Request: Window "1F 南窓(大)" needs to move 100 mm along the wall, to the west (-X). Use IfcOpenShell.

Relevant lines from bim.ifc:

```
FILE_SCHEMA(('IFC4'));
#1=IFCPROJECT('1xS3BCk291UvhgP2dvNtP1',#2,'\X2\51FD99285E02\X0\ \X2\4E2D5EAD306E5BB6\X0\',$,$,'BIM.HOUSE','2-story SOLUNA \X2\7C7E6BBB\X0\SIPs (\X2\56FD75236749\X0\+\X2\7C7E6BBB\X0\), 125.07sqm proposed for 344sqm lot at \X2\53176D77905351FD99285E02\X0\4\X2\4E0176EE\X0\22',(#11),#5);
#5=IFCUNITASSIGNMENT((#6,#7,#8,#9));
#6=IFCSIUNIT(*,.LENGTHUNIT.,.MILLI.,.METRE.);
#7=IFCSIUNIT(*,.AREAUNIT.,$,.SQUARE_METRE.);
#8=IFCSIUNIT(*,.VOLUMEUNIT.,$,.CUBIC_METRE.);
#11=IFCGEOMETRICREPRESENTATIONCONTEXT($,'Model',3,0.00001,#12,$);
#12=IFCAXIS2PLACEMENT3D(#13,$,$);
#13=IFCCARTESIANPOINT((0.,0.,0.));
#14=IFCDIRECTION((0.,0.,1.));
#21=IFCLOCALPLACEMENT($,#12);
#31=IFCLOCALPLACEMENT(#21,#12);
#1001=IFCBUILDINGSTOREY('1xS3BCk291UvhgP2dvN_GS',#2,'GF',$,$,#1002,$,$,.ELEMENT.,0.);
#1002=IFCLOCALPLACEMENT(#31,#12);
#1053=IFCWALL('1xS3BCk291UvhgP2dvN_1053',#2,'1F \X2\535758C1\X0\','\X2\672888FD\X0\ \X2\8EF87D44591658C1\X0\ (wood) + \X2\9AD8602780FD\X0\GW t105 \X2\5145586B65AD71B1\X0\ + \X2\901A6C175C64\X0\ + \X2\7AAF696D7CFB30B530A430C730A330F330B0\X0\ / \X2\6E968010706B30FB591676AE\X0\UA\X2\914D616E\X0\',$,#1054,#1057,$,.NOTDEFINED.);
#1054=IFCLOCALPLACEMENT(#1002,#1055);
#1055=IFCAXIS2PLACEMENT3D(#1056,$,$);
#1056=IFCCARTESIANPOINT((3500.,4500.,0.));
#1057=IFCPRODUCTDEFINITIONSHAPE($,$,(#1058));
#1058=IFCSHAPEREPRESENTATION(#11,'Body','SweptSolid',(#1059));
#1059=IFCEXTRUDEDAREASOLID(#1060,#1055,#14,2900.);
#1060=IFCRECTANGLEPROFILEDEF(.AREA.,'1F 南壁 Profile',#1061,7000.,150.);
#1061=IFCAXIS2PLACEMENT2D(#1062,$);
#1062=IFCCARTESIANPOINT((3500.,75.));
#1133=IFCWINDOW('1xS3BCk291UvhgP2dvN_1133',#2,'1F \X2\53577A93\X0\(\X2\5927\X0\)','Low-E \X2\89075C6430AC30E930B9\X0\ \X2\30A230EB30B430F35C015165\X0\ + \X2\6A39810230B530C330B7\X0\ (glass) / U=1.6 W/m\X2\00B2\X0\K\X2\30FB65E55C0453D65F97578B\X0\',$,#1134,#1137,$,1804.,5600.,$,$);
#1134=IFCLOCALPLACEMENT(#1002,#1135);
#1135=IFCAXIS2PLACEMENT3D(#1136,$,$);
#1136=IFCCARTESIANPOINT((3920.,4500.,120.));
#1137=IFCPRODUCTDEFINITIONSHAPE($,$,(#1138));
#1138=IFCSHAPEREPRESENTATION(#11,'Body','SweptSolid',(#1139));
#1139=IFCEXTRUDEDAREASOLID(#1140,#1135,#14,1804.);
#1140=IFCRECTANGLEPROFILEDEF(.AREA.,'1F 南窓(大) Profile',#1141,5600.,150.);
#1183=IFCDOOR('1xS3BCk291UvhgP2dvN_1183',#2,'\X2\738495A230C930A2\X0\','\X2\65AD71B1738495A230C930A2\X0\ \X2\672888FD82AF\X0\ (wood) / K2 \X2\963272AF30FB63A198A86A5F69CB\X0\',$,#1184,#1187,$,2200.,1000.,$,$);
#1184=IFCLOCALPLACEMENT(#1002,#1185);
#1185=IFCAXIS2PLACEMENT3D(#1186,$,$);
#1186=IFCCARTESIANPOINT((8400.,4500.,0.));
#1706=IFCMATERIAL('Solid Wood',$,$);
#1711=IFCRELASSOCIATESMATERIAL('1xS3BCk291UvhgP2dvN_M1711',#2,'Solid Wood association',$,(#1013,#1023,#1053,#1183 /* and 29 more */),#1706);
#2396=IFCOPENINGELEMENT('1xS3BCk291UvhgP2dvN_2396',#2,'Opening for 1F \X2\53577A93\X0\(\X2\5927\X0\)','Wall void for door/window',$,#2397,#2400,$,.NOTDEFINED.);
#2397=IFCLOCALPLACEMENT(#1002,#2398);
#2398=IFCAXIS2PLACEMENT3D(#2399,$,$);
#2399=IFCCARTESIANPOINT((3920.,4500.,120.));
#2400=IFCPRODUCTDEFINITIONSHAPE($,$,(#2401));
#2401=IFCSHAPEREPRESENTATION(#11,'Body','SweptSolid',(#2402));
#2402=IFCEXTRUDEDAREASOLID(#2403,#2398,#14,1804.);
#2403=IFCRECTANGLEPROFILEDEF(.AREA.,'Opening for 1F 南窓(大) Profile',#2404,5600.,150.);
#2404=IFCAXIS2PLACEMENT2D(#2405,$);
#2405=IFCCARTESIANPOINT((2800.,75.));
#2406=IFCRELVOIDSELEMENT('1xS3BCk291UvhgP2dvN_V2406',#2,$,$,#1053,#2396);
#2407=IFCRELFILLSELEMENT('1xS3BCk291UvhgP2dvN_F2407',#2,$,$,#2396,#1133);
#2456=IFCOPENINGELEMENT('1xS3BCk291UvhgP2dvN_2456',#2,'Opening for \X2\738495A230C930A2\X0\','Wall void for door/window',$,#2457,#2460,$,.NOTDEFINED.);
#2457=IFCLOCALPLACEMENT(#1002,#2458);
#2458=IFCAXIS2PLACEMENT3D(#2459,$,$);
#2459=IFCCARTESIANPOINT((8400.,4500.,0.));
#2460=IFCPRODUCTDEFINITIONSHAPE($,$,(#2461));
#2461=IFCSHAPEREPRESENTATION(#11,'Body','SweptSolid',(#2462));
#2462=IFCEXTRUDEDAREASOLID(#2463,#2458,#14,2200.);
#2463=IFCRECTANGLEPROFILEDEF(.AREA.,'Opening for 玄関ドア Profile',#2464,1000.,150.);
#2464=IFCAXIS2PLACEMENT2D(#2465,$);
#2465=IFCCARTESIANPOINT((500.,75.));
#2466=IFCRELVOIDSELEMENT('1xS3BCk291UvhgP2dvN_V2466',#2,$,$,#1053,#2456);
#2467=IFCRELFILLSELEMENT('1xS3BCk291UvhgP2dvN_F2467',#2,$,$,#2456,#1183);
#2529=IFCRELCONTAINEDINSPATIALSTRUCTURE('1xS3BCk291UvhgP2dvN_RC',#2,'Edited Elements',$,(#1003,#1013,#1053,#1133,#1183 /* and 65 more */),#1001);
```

```python
import ifcopenshell
import ifcopenshell.api.geometry
import ifcopenshell.util.placement
import ifcopenshell.util.unit

model = ifcopenshell.open("bim.ifc")
unit_scale = ifcopenshell.util.unit.calculate_unit_scale(model)

window = model.by_guid("1xS3BCk291UvhgP2dvN_1133")
opening = window.FillsVoids[0].RelatingOpeningElement
wall = opening.VoidsElements[0].RelatingBuildingElement

wall_matrix = ifcopenshell.util.placement.get_local_placement(wall.ObjectPlacement)
shift = wall_matrix[:3, 0] * -0.1 / unit_scale
before = ifcopenshell.util.placement.get_local_placement(window.ObjectPlacement)[:3, 3].copy()

# The window is not placed relative to its opening, so move both.
for product in (opening, window):
    matrix = ifcopenshell.util.placement.get_local_placement(product.ObjectPlacement)
    matrix[:3, 3] += shift
    ifcopenshell.api.geometry.edit_object_placement(model, product=product, matrix=matrix, is_si=False)

after = ifcopenshell.util.placement.get_local_placement(window.ObjectPlacement)[:3, 3]
print("window moved by", (after - before).round(3) + 0.0)

model.write("bim_v2.ifc")
```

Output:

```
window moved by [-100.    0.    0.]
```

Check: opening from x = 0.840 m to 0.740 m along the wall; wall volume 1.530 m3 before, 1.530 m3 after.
